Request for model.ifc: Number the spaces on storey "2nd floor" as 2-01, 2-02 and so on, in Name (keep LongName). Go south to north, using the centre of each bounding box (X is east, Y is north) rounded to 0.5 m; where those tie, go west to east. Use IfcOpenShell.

First a look at what the model holds.

```python
import ifcopenshell
import ifcopenshell.util.element
import ifcopenshell.util.placement

model = ifcopenshell.open("model.ifc")
print(model.schema)
storey = next(s for s in model.by_type("IfcBuildingStorey") if s.Name == "2nd floor")
spaces = [e for e in ifcopenshell.util.element.get_decomposition(storey) if e.is_a("IfcSpace")]
for e in sorted(spaces, key=lambda e: e.id()):
    origin = ifcopenshell.util.placement.get_local_placement(e.ObjectPlacement)[:3, 3]
    print(e.id(), e.Name, e.LongName, origin.round(2) + 0.0, sep=" | ")
```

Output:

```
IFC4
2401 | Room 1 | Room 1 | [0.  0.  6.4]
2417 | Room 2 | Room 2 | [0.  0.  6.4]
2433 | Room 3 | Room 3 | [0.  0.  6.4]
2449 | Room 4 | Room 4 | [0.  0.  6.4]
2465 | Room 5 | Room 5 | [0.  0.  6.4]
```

```python
import ifcopenshell
import ifcopenshell.geom
import ifcopenshell.util.element
import ifcopenshell.util.shape

model = ifcopenshell.open("model.ifc")
settings = ifcopenshell.geom.settings()
settings.set("use-world-coords", True)


def centre(element):
    shape = ifcopenshell.geom.create_shape(settings, element)
    return ifcopenshell.util.shape.get_bbox_centroid(shape.geometry)


storey = next(s for s in model.by_type("IfcBuildingStorey") if s.Name == "2nd floor")
spaces = [e for e in ifcopenshell.util.element.get_decomposition(storey) if e.is_a("IfcSpace")]

# Insertion points can sit at a corner or the storey origin, so sort by the geometry (in metres).
centres = {e: centre(e) for e in spaces}
spaces.sort(key=lambda e: (round(centres[e][1] / 0.5), centres[e][0]))

for i, e in enumerate(spaces, start=1):
    number = f"2-{i:02d}"
    e.Name = number
    print(e.id(), number)

model.write("model_v2.ifc")
```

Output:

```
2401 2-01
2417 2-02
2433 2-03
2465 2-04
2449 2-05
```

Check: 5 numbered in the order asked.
